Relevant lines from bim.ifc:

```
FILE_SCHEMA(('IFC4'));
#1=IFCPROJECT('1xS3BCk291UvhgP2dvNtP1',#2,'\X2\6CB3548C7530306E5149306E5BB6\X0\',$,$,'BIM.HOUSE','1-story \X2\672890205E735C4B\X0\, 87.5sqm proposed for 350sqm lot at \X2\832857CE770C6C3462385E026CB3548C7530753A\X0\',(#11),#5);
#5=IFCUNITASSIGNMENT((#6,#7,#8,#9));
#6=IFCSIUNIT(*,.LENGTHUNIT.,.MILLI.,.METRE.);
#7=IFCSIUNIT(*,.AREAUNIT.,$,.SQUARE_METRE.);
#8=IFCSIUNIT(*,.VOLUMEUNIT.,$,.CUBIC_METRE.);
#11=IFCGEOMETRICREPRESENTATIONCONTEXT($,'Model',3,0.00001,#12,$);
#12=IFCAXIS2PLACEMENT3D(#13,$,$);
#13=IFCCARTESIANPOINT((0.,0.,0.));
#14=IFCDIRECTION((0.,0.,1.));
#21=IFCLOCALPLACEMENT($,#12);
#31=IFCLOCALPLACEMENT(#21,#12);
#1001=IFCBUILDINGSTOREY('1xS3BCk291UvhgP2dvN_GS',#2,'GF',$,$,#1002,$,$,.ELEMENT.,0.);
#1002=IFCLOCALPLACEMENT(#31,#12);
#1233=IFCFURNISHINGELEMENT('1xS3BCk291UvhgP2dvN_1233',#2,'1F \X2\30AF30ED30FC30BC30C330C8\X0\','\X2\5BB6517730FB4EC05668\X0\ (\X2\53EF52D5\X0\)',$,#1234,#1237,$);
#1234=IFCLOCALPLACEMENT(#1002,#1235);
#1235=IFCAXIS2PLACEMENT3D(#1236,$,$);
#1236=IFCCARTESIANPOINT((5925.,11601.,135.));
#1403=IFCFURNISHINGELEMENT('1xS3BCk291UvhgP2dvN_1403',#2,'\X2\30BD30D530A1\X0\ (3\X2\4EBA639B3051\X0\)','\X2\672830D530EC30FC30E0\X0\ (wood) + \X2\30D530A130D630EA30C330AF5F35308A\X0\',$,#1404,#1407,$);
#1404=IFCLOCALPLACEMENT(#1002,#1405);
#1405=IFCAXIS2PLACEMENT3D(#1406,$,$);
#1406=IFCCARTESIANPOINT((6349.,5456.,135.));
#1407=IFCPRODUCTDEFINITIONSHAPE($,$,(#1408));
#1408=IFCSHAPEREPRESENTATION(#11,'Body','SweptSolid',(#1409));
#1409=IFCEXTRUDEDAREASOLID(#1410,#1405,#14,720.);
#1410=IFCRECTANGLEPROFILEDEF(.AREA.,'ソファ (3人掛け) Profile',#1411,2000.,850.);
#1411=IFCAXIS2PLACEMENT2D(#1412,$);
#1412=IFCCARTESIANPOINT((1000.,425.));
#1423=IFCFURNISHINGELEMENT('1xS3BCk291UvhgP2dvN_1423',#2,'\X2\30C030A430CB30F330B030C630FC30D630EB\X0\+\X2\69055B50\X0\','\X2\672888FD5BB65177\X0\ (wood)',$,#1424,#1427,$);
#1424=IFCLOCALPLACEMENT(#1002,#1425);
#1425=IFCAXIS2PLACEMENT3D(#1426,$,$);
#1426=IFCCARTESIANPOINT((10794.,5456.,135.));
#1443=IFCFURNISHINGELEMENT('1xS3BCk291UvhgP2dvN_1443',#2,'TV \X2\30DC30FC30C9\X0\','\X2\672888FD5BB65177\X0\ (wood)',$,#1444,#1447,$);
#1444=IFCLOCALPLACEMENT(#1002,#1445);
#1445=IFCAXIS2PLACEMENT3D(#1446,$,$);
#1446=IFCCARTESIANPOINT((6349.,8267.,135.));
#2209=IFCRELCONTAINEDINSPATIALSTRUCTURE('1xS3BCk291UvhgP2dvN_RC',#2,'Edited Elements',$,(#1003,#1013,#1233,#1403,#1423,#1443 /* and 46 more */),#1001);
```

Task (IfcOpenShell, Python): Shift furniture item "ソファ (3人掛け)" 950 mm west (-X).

```python
import ifcopenshell
import ifcopenshell.api.geometry
import ifcopenshell.util.placement
import ifcopenshell.util.unit

model = ifcopenshell.open("bim.ifc")
unit_scale = ifcopenshell.util.unit.calculate_unit_scale(model)

item = model.by_guid("1xS3BCk291UvhgP2dvN_1403")
matrix = ifcopenshell.util.placement.get_local_placement(item.ObjectPlacement)
matrix[0, 3] -= 0.95 / unit_scale
ifcopenshell.api.geometry.edit_object_placement(model, product=item, matrix=matrix, is_si=False)

print(ifcopenshell.util.placement.get_local_placement(item.ObjectPlacement).round(3) + 0.0)

model.write("bim_edited.ifc")
```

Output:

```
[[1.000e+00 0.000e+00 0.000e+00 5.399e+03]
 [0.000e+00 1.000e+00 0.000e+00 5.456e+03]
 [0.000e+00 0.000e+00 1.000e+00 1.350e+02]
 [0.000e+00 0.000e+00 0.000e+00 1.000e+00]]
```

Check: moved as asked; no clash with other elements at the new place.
